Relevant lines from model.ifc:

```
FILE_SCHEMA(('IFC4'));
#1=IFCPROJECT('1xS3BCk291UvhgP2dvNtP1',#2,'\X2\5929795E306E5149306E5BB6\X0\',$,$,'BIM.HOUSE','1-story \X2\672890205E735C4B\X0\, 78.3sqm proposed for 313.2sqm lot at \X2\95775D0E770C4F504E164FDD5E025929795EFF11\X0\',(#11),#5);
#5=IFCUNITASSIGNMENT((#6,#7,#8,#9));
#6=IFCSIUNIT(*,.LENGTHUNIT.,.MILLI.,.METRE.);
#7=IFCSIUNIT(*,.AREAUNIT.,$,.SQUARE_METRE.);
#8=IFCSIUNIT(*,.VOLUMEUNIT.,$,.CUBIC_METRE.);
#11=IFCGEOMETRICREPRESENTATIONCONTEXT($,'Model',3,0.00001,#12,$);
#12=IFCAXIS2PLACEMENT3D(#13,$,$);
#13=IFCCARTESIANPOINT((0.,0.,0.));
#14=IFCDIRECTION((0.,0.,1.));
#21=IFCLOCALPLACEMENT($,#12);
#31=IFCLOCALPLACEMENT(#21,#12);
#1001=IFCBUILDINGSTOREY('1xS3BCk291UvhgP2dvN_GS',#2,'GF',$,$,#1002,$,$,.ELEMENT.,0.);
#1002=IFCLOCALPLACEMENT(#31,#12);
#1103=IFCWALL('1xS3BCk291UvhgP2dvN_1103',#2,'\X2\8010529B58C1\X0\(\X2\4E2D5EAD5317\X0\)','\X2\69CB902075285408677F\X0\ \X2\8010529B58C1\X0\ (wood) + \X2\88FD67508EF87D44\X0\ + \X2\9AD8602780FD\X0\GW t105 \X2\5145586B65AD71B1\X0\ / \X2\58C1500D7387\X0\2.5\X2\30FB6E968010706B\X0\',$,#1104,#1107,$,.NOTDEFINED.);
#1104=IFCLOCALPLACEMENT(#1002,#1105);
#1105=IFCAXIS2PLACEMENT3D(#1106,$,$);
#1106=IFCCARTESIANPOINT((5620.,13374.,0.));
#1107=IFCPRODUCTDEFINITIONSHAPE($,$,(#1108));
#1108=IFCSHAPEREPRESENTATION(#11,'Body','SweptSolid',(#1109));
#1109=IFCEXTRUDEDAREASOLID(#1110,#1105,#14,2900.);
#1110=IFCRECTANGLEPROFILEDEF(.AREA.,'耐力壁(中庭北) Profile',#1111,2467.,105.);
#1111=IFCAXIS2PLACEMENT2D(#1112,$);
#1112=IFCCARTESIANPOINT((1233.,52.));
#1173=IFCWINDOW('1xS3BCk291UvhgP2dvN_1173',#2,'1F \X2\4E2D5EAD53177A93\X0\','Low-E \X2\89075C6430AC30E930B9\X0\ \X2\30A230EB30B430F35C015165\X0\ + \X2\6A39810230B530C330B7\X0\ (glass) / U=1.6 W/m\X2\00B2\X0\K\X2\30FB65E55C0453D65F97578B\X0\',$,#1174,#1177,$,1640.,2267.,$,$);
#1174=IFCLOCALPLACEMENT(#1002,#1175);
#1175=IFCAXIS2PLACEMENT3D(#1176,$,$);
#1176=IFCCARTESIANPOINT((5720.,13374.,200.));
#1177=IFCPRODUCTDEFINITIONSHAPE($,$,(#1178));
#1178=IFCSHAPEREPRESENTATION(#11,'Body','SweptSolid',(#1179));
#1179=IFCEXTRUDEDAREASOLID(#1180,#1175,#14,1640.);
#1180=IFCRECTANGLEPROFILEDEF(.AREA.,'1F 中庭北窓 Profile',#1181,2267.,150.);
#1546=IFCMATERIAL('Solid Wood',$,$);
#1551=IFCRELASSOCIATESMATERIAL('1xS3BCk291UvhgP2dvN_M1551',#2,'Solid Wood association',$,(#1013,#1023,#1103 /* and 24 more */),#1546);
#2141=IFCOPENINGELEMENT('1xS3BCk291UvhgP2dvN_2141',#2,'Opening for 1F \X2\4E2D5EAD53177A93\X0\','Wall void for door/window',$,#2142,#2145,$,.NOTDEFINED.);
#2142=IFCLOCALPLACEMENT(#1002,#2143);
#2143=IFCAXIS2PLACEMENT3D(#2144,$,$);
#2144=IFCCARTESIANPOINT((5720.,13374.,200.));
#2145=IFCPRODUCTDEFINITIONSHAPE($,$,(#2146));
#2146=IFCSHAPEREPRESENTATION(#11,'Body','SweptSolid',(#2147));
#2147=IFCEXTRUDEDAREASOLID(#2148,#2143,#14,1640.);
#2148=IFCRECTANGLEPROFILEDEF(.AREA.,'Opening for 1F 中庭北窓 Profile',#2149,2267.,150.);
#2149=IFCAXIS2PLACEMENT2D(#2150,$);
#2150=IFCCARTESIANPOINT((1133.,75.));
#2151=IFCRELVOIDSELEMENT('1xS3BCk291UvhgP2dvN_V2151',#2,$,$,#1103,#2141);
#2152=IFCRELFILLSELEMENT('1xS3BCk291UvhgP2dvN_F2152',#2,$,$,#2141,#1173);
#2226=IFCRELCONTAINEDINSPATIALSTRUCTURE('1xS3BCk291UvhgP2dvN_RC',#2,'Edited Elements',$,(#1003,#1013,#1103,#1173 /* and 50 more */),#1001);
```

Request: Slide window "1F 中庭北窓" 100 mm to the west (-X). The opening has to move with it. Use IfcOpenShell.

```python
import ifcopenshell
import ifcopenshell.api.geometry
import ifcopenshell.util.placement
import ifcopenshell.util.unit

model = ifcopenshell.open("model.ifc")
unit_scale = ifcopenshell.util.unit.calculate_unit_scale(model)

window = model.by_guid("1xS3BCk291UvhgP2dvN_1173")
opening = window.FillsVoids[0].RelatingOpeningElement
wall = opening.VoidsElements[0].RelatingBuildingElement

wall_matrix = ifcopenshell.util.placement.get_local_placement(wall.ObjectPlacement)
shift = wall_matrix[:3, 0] * -0.1 / unit_scale
before = ifcopenshell.util.placement.get_local_placement(window.ObjectPlacement)[:3, 3].copy()

# The window is not placed relative to its opening, so move both.
for product in (opening, window):
    matrix = ifcopenshell.util.placement.get_local_placement(product.ObjectPlacement)
    matrix[:3, 3] += shift
    ifcopenshell.api.geometry.edit_object_placement(model, product=product, matrix=matrix, is_si=False)

after = ifcopenshell.util.placement.get_local_placement(window.ObjectPlacement)[:3, 3]
print("window moved by", (after - before).round(3) + 0.0)

model.write("model_updated.ifc")
```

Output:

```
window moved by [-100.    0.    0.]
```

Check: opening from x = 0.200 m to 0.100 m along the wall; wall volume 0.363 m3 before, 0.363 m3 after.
